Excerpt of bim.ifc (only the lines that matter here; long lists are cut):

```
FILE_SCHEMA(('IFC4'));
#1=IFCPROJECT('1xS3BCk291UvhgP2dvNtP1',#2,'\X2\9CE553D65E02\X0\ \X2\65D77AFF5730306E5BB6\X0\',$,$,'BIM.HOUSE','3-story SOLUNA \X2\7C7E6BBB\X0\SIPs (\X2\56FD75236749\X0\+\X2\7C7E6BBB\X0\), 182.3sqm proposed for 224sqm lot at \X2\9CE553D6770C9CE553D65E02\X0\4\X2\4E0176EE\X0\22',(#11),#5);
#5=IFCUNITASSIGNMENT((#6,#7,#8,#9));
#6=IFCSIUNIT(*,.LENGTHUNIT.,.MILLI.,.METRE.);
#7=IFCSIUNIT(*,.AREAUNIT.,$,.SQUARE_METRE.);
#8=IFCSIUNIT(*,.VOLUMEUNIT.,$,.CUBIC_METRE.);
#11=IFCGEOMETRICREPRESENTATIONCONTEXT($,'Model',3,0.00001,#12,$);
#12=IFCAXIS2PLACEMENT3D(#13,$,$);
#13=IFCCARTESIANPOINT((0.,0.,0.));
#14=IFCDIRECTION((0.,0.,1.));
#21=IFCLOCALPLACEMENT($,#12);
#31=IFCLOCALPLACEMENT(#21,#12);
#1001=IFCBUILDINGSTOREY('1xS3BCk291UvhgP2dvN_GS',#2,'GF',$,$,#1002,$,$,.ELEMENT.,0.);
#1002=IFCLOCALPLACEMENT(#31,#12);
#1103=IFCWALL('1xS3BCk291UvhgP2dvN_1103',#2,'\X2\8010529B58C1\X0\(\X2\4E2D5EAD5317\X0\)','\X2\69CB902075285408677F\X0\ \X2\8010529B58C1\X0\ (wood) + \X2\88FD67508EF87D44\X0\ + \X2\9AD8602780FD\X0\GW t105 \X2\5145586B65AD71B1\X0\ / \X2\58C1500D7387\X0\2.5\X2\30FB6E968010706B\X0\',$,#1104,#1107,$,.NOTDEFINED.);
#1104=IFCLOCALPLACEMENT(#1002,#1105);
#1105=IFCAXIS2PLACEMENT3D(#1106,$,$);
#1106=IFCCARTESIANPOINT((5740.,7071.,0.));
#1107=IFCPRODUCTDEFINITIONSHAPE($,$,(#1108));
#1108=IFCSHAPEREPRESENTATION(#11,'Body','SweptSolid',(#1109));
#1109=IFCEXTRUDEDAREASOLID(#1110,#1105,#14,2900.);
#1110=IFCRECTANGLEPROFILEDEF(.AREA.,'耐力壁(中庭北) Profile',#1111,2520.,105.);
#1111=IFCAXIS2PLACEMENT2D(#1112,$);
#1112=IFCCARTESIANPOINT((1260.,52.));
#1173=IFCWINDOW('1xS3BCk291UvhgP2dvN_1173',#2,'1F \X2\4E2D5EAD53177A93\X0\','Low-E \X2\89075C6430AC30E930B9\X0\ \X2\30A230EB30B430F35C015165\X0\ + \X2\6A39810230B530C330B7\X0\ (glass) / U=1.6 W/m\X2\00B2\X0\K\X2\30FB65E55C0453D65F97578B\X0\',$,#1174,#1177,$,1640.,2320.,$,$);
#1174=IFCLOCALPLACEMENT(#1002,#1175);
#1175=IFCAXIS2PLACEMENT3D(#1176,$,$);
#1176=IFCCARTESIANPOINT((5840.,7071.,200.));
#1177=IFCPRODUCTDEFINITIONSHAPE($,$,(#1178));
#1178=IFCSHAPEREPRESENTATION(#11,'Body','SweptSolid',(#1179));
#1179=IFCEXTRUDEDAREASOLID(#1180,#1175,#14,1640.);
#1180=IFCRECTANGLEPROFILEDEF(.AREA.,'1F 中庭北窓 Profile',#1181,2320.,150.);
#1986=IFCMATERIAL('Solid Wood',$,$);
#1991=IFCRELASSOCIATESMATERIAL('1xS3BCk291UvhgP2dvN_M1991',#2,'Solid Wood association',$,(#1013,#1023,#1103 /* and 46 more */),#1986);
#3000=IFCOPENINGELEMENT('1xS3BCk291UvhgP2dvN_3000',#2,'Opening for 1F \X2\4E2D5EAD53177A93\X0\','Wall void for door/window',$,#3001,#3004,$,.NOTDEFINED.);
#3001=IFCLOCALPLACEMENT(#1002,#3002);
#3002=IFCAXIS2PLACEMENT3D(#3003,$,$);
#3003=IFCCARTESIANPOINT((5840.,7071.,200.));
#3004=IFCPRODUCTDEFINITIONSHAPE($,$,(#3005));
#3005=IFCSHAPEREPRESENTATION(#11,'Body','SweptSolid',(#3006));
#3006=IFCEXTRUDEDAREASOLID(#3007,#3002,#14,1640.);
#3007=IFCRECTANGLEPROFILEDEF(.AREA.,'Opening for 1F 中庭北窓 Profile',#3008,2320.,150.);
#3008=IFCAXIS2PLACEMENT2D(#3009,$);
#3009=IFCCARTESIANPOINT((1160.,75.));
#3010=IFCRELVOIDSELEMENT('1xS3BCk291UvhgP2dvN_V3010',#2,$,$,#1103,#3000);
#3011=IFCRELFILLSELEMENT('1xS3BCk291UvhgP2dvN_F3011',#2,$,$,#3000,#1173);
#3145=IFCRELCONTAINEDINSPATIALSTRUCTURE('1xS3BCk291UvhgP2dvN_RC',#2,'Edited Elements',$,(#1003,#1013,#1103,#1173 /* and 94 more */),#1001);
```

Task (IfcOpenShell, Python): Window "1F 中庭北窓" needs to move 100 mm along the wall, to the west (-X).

```python
import ifcopenshell
import ifcopenshell.api.geometry
import ifcopenshell.util.placement
import ifcopenshell.util.unit

model = ifcopenshell.open("bim.ifc")
unit_scale = ifcopenshell.util.unit.calculate_unit_scale(model)

window = model.by_guid("1xS3BCk291UvhgP2dvN_1173")
opening = window.FillsVoids[0].RelatingOpeningElement
wall = opening.VoidsElements[0].RelatingBuildingElement

wall_matrix = ifcopenshell.util.placement.get_local_placement(wall.ObjectPlacement)
shift = wall_matrix[:3, 0] * -0.1 / unit_scale
before = ifcopenshell.util.placement.get_local_placement(window.ObjectPlacement)[:3, 3].copy()

# The window is not placed relative to its opening, so move both.
for product in (opening, window):
    matrix = ifcopenshell.util.placement.get_local_placement(product.ObjectPlacement)
    matrix[:3, 3] += shift
    ifcopenshell.api.geometry.edit_object_placement(model, product=product, matrix=matrix, is_si=False)

after = ifcopenshell.util.placement.get_local_placement(window.ObjectPlacement)[:3, 3]
print("window moved by", (after - before).round(3) + 0.0)

model.write("bim_edited.ifc")
```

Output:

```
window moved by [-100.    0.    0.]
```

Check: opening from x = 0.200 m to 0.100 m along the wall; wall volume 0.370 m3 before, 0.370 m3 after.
